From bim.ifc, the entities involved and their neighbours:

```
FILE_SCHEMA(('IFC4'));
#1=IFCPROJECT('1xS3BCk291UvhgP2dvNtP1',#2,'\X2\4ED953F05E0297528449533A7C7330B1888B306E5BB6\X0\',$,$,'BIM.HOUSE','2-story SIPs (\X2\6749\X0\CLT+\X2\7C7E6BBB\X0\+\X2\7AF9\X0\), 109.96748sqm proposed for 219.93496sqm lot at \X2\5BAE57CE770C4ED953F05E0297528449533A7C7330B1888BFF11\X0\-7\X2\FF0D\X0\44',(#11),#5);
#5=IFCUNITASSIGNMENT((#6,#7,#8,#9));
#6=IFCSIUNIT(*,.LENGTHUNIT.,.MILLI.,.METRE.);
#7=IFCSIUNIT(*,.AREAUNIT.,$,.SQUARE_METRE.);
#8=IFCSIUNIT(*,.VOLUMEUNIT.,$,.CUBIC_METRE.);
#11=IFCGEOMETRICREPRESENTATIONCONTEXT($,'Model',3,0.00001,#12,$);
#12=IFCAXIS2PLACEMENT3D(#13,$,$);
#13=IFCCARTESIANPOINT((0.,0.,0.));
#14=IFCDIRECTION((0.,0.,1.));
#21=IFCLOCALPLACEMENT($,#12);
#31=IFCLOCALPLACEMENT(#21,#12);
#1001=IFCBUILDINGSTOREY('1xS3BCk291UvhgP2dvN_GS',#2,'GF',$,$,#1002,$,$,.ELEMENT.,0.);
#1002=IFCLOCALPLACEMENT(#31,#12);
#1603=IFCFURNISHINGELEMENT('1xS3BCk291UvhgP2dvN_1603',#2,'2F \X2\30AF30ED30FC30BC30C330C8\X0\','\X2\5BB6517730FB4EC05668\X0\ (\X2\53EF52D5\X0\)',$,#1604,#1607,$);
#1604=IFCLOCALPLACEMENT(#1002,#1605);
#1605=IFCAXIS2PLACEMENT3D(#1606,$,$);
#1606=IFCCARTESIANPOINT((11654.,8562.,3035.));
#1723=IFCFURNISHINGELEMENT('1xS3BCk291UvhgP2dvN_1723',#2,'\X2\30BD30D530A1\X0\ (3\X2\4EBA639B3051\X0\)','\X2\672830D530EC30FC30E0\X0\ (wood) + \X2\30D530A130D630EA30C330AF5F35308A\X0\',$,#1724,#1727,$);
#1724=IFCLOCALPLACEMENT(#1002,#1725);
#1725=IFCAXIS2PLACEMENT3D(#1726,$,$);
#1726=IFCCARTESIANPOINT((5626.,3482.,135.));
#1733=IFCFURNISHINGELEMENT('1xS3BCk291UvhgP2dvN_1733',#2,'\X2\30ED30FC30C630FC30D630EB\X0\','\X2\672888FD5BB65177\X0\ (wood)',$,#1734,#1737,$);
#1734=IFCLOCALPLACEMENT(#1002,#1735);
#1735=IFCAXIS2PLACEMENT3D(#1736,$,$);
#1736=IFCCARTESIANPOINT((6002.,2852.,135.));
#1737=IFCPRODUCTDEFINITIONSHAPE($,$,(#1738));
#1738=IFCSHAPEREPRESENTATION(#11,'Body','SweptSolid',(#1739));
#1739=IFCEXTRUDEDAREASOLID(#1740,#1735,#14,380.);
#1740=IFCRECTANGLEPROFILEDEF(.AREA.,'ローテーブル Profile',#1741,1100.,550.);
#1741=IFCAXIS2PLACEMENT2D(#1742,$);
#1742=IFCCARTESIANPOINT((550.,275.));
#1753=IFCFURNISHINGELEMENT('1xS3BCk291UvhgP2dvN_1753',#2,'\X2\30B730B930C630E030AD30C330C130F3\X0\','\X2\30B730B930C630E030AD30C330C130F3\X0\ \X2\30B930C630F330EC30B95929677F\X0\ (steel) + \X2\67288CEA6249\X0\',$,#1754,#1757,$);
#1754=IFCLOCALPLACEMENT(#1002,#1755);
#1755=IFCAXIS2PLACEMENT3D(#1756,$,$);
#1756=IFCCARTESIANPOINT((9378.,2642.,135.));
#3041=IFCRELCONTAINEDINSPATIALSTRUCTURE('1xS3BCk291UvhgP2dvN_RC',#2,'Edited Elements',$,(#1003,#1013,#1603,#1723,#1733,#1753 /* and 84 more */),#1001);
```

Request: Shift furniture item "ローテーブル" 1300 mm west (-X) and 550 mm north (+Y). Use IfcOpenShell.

```python
import ifcopenshell
import ifcopenshell.api.geometry
import ifcopenshell.util.placement

model = ifcopenshell.open("bim.ifc")

item = model.by_guid("1xS3BCk291UvhgP2dvN_1733")
matrix = ifcopenshell.util.placement.get_local_placement(item.ObjectPlacement)
matrix[0, 3] -= 1300.0
matrix[1, 3] += 550.0
ifcopenshell.api.geometry.edit_object_placement(model, product=item, matrix=matrix, is_si=False)

print(ifcopenshell.util.placement.get_local_placement(item.ObjectPlacement).round(3) + 0.0)

model.write("bim_edited.ifc")
```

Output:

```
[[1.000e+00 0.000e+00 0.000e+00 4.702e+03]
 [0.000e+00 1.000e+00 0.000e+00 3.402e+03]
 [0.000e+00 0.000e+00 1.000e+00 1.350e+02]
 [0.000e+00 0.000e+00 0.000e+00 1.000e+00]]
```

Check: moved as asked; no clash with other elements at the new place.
